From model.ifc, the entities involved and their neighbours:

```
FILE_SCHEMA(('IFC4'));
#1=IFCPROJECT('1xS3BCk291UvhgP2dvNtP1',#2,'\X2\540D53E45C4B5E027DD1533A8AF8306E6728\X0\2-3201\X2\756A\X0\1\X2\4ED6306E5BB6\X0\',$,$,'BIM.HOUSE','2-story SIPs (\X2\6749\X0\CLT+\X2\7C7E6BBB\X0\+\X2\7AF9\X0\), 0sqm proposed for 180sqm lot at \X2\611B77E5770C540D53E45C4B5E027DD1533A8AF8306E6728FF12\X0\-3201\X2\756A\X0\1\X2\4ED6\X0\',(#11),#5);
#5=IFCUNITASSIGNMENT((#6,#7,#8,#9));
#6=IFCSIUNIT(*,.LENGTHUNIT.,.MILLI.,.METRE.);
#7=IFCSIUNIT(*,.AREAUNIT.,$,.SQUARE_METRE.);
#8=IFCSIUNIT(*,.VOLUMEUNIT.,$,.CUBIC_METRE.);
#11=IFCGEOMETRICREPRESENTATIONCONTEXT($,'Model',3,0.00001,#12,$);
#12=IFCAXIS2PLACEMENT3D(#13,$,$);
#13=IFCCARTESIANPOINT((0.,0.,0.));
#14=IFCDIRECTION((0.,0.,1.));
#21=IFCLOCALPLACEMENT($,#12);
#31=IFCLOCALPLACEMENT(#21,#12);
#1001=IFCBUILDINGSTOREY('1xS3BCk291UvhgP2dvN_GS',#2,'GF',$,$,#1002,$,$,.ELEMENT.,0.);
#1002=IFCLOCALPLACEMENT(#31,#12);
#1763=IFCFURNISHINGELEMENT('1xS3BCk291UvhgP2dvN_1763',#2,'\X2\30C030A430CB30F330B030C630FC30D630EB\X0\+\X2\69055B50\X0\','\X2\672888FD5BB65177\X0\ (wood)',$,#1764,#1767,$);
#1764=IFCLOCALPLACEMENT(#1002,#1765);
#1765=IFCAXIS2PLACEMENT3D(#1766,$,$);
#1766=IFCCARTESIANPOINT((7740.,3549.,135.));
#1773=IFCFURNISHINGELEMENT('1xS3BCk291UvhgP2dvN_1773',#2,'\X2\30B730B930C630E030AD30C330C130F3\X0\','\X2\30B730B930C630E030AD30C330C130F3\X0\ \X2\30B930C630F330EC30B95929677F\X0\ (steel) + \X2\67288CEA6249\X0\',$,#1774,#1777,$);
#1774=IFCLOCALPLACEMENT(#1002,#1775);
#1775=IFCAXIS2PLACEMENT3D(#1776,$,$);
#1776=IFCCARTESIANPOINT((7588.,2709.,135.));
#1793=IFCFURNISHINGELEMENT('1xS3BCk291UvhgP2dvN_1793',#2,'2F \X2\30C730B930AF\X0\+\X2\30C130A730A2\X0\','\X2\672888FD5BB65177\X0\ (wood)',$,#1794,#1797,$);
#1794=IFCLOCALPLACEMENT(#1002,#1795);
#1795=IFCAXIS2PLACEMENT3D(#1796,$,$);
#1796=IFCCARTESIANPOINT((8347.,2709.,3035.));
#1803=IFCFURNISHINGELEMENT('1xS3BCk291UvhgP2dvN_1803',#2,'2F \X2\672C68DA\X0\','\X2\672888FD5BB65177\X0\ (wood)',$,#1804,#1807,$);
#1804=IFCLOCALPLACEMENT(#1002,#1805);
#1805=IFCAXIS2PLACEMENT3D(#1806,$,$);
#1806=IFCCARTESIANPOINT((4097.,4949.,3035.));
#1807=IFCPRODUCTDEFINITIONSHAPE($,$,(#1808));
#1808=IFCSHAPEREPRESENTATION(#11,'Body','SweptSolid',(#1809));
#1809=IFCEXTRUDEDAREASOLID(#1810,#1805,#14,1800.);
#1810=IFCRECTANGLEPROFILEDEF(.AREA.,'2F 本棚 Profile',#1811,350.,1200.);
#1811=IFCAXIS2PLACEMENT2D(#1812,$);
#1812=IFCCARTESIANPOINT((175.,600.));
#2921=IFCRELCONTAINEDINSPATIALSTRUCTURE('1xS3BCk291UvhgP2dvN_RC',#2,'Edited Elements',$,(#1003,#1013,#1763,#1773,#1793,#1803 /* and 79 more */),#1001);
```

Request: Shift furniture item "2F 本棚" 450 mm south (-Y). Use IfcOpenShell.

```python
import ifcopenshell
import ifcopenshell.api.geometry
import ifcopenshell.util.placement

model = ifcopenshell.open("model.ifc")

item = model.by_id(1803)
matrix = ifcopenshell.util.placement.get_local_placement(item.ObjectPlacement)
matrix[1, 3] -= 450.0
ifcopenshell.api.geometry.edit_object_placement(model, product=item, matrix=matrix, is_si=False)

print(ifcopenshell.util.placement.get_local_placement(item.ObjectPlacement).round(3) + 0.0)

model.write("model_rev.ifc")
```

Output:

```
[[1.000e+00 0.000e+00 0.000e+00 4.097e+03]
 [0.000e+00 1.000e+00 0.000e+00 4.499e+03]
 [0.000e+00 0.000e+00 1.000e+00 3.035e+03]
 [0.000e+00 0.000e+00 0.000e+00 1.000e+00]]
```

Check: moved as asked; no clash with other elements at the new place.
